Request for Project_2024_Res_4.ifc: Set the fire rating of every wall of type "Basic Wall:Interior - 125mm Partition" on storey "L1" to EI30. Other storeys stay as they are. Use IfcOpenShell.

First a look at what the model holds.

```python
import ifcopenshell
import ifcopenshell.util.element

model = ifcopenshell.open("Project_2024_Res_4.ifc")
print(model.schema)
storey = next(s for s in model.by_type("IfcBuildingStorey") if s.Name == "L1")
walls = [e for e in ifcopenshell.util.element.get_decomposition(storey) if e.is_a("IfcWall")]
seen = {}
for e in walls:
    element_type = ifcopenshell.util.element.get_type(e)
    key = (element_type.Name if element_type != e and element_type else None, ifcopenshell.util.element.get_pset(e, "Pset_WallCommon", "FireRating"))
    seen[key] = seen.get(key, 0) + 1
for (name, value), count in sorted(seen.items(), key=str):
    print(count, "x", name, "|", value)
```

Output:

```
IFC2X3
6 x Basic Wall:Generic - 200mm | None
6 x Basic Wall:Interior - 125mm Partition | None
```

```python
import ifcopenshell
import ifcopenshell.api.pset
import ifcopenshell.util.element

model = ifcopenshell.open("Project_2024_Res_4.ifc")

storey = next(s for s in model.by_type("IfcBuildingStorey") if s.Name == "L1")
walls = [e for e in ifcopenshell.util.element.get_decomposition(storey) if e.is_a("IfcWall")]

count = 0
for e in walls:
    element_type = ifcopenshell.util.element.get_type(e)
    if element_type in (None, e) or element_type.Name != "Basic Wall:Interior - 125mm Partition":
        continue
    # add_pset returns the element's existing set when there is one.
    pset = ifcopenshell.api.pset.add_pset(model, product=e, name="Pset_WallCommon")
    ifcopenshell.api.pset.edit_pset(model, pset=pset, properties={"FireRating": "EI30"})
    count += 1

print(count, "walls updated")

model.write("Project_2024_Res_4_updated.ifc")
```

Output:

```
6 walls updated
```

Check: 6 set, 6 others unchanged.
